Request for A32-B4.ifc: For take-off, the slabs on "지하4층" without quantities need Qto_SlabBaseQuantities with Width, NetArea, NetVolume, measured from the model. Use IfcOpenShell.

First a look at what the model holds.

```python
import ifcopenshell
import ifcopenshell.util.element
import ifcopenshell.util.unit

model = ifcopenshell.open("A32-B4.ifc")
print(model.schema)
for unit_type in ("LENGTHUNIT", "AREAUNIT", "VOLUMEUNIT"):
    print(unit_type, ifcopenshell.util.unit.calculate_unit_scale(model, unit_type))
storey = next(s for s in model.by_type("IfcBuildingStorey") if s.Name == "지하4층")
slabs = [e for e in ifcopenshell.util.element.get_decomposition(storey) if e.is_a("IfcSlab")]
for e in sorted(slabs, key=lambda e: e.id()):
    print(e.id(), e.is_a(), e.Name, list(ifcopenshell.util.element.get_psets(e, qtos_only=True)), sep=" | ")
```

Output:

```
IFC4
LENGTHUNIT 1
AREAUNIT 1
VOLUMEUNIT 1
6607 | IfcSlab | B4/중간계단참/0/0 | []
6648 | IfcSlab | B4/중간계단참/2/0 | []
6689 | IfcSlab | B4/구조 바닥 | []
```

```python
import ifcopenshell
import ifcopenshell.api.pset
import ifcopenshell.geom
import ifcopenshell.util.element
import ifcopenshell.util.shape
import ifcopenshell.util.unit

model = ifcopenshell.open("A32-B4.ifc")
unit_scale = ifcopenshell.util.unit.calculate_unit_scale(model)
area_scale = ifcopenshell.util.unit.calculate_unit_scale(model, "AREAUNIT")
volume_scale = ifcopenshell.util.unit.calculate_unit_scale(model, "VOLUMEUNIT")
settings = ifcopenshell.geom.settings()

storey = next(s for s in model.by_type("IfcBuildingStorey") if s.Name == "지하4층")
slabs = [e for e in ifcopenshell.util.element.get_decomposition(storey) if e.is_a("IfcSlab")]

for e in sorted(slabs, key=lambda e: e.id()):
    if ifcopenshell.util.element.get_psets(e, qtos_only=True, should_inherit=False):
        continue
    # Geometry comes back in metres, in the element's own axes.
    shape = ifcopenshell.geom.create_shape(settings, e)
    values = {
        "Width": ifcopenshell.util.shape.get_z(shape.geometry) / unit_scale,
        "NetArea": ifcopenshell.util.shape.get_footprint_area(shape.geometry) / area_scale,
        "NetVolume": ifcopenshell.util.shape.get_volume(shape.geometry) / volume_scale,
    }
    qto = ifcopenshell.api.pset.add_qto(model, product=e, name="Qto_SlabBaseQuantities")
    ifcopenshell.api.pset.edit_qto(model, qto=qto, properties=values)
    print(e.id(), {k: round(v, 3) for k, v in values.items()})

model.write("A32-B4_edited.ifc")
```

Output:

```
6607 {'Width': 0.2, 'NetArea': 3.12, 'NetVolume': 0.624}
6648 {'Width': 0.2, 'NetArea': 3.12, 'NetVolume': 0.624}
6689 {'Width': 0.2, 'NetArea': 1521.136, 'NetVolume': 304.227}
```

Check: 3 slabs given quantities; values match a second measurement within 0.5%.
